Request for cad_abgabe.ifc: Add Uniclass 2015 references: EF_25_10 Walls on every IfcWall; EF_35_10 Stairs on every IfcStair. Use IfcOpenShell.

First a look at what the model holds.

```python
import ifcopenshell

model = ifcopenshell.open("cad_abgabe.ifc")
print(model.schema)
print("classifications:", [c.Name for c in model.by_type("IfcClassification")])
for ifc_class in ("IfcDoor", "IfcRoof", "IfcStair", "IfcWall", "IfcWindow"):
    print(ifc_class, len(model.by_type(ifc_class)))
```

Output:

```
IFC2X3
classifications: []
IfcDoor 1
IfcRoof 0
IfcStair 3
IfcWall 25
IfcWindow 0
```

```python
import ifcopenshell
import ifcopenshell.api.classification

model = ifcopenshell.open("cad_abgabe.ifc")

# IFC2X3 requires Source and Edition and has no link from the project to the system.
system = model.create_entity("IfcClassification", Source="NBS", Edition="2015", Name="Uniclass 2015")

codes = {
    "IfcWall": ("EF_25_10", "Walls"),
    "IfcStair": ("EF_35_10", "Stairs"),
}
for ifc_class, (code, name) in codes.items():
    products = model.by_type(ifc_class)
    ifcopenshell.api.classification.add_reference(
        model, products=products, classification=system, identification=code, name=name
    )
    print(code, len(products))

model.write("cad_abgabe_edited.ifc")
```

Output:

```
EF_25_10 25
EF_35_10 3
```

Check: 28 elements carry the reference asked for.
